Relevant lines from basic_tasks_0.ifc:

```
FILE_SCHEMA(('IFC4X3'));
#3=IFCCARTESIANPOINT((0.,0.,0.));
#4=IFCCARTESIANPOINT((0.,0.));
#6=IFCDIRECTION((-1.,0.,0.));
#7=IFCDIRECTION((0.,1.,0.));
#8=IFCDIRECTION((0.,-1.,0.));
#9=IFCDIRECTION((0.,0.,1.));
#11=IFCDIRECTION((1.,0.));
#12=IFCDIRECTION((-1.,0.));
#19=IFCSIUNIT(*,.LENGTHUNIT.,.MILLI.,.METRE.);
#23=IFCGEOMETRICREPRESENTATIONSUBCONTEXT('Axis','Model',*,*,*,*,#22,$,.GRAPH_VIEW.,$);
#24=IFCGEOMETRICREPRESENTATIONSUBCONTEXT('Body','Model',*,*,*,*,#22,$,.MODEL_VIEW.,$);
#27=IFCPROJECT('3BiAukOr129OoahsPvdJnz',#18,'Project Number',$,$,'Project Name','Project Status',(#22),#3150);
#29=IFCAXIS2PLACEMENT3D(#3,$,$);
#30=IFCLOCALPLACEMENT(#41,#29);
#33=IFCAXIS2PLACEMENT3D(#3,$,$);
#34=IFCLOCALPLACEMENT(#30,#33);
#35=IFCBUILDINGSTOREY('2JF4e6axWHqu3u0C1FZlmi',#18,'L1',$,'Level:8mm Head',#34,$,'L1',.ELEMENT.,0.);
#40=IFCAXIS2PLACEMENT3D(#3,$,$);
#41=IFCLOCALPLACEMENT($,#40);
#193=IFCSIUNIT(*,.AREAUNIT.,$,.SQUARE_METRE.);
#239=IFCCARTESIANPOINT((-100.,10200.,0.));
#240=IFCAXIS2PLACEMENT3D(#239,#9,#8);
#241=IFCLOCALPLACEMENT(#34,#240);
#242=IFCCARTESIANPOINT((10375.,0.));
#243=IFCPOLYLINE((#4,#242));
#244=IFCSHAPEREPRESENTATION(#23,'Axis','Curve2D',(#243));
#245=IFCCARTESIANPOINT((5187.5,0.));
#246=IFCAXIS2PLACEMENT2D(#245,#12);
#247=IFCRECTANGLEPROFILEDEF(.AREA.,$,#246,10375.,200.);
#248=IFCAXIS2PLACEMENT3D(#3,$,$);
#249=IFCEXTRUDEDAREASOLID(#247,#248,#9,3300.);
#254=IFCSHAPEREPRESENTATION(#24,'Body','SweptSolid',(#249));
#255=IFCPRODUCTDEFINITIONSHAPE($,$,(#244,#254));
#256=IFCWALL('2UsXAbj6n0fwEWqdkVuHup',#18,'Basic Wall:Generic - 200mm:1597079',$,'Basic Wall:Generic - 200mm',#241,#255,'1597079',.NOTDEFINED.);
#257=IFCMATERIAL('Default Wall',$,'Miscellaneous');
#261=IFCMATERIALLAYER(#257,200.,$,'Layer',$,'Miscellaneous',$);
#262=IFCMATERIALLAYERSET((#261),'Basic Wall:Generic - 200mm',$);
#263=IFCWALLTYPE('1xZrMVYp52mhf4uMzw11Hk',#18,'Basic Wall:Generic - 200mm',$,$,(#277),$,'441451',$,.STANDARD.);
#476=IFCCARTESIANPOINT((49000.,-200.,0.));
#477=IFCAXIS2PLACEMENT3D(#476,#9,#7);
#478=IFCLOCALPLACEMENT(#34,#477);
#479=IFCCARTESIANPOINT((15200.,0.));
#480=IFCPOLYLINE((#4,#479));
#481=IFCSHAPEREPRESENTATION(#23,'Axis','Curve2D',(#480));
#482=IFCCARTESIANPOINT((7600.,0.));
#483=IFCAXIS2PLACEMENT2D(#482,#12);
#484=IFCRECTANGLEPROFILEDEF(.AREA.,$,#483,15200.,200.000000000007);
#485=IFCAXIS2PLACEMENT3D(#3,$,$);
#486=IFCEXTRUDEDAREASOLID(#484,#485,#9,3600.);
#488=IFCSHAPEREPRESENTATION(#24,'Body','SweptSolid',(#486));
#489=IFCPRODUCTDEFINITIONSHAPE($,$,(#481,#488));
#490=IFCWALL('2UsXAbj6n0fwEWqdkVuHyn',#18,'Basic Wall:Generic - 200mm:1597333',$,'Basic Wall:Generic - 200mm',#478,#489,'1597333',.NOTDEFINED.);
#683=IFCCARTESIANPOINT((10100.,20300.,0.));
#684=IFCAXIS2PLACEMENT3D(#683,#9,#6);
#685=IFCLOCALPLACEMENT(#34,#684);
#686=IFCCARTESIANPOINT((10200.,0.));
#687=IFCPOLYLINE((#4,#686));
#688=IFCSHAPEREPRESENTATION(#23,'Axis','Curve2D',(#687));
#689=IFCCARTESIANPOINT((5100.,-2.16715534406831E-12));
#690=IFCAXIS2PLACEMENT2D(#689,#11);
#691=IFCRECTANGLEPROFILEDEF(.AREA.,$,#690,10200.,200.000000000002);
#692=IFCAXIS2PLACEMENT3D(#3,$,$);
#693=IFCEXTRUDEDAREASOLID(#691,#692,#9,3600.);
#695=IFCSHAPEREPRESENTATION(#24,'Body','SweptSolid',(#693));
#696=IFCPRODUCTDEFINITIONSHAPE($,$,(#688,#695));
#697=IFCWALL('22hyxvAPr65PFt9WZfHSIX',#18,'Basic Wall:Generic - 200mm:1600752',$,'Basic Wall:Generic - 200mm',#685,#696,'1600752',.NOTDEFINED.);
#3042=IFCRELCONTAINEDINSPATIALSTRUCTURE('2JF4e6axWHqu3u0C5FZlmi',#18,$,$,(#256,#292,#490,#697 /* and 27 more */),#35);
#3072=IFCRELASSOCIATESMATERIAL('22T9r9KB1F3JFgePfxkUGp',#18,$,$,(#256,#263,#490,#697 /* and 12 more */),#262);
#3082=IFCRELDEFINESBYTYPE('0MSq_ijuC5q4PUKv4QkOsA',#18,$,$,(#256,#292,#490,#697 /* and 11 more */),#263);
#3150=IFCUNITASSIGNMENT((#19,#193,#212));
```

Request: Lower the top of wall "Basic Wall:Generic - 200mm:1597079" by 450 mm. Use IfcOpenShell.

```python
import ifcopenshell
import ifcopenshell.geom
import ifcopenshell.util.representation
import ifcopenshell.util.shape
import ifcopenshell.util.unit

model = ifcopenshell.open("basic_tasks_0.ifc")
unit_scale = ifcopenshell.util.unit.calculate_unit_scale(model)
settings = ifcopenshell.geom.settings()


def volume(element):
    """Net volume in cubic metres, openings subtracted."""
    shape = ifcopenshell.geom.create_shape(settings, element)
    return ifcopenshell.util.shape.get_volume(shape.geometry)


wall = model.by_guid("2UsXAbj6n0fwEWqdkVuHup")
before = volume(wall)

body = ifcopenshell.util.representation.get_representation(wall, "Model", "Body")
solid = body.Items[0]
old_height = solid.Depth
solid.Depth -= 0.45 / unit_scale
after = volume(wall)

print(f"height {old_height:g} -> {solid.Depth:g}, volume {before:.3f} -> {after:.3f} m3")

model.write("basic_tasks_0_v2.ifc")
```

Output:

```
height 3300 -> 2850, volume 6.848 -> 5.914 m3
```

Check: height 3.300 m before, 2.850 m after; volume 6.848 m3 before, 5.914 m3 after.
